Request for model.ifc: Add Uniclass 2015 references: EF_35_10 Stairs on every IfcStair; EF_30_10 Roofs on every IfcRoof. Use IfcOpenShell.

First a look at what the model holds.

```python
import ifcopenshell

model = ifcopenshell.open("model.ifc")
print(model.schema)
print("classifications:", [c.Name for c in model.by_type("IfcClassification")])
for ifc_class in ("IfcDoor", "IfcRoof", "IfcStair", "IfcWall", "IfcWindow"):
    print(ifc_class, len(model.by_type(ifc_class)))
```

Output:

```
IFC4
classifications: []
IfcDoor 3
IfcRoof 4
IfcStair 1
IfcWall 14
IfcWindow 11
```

```python
import ifcopenshell
import ifcopenshell.api.classification

model = ifcopenshell.open("model.ifc")

system = ifcopenshell.api.classification.add_classification(model, classification="Uniclass 2015")

codes = {
    "IfcStair": ("EF_35_10", "Stairs"),
    "IfcRoof": ("EF_30_10", "Roofs"),
}
for ifc_class, (code, name) in codes.items():
    products = model.by_type(ifc_class)
    ifcopenshell.api.classification.add_reference(
        model, products=products, classification=system, identification=code, name=name
    )
    print(code, len(products))

model.write("model_rev.ifc")
```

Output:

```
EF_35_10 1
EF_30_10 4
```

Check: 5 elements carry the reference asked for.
